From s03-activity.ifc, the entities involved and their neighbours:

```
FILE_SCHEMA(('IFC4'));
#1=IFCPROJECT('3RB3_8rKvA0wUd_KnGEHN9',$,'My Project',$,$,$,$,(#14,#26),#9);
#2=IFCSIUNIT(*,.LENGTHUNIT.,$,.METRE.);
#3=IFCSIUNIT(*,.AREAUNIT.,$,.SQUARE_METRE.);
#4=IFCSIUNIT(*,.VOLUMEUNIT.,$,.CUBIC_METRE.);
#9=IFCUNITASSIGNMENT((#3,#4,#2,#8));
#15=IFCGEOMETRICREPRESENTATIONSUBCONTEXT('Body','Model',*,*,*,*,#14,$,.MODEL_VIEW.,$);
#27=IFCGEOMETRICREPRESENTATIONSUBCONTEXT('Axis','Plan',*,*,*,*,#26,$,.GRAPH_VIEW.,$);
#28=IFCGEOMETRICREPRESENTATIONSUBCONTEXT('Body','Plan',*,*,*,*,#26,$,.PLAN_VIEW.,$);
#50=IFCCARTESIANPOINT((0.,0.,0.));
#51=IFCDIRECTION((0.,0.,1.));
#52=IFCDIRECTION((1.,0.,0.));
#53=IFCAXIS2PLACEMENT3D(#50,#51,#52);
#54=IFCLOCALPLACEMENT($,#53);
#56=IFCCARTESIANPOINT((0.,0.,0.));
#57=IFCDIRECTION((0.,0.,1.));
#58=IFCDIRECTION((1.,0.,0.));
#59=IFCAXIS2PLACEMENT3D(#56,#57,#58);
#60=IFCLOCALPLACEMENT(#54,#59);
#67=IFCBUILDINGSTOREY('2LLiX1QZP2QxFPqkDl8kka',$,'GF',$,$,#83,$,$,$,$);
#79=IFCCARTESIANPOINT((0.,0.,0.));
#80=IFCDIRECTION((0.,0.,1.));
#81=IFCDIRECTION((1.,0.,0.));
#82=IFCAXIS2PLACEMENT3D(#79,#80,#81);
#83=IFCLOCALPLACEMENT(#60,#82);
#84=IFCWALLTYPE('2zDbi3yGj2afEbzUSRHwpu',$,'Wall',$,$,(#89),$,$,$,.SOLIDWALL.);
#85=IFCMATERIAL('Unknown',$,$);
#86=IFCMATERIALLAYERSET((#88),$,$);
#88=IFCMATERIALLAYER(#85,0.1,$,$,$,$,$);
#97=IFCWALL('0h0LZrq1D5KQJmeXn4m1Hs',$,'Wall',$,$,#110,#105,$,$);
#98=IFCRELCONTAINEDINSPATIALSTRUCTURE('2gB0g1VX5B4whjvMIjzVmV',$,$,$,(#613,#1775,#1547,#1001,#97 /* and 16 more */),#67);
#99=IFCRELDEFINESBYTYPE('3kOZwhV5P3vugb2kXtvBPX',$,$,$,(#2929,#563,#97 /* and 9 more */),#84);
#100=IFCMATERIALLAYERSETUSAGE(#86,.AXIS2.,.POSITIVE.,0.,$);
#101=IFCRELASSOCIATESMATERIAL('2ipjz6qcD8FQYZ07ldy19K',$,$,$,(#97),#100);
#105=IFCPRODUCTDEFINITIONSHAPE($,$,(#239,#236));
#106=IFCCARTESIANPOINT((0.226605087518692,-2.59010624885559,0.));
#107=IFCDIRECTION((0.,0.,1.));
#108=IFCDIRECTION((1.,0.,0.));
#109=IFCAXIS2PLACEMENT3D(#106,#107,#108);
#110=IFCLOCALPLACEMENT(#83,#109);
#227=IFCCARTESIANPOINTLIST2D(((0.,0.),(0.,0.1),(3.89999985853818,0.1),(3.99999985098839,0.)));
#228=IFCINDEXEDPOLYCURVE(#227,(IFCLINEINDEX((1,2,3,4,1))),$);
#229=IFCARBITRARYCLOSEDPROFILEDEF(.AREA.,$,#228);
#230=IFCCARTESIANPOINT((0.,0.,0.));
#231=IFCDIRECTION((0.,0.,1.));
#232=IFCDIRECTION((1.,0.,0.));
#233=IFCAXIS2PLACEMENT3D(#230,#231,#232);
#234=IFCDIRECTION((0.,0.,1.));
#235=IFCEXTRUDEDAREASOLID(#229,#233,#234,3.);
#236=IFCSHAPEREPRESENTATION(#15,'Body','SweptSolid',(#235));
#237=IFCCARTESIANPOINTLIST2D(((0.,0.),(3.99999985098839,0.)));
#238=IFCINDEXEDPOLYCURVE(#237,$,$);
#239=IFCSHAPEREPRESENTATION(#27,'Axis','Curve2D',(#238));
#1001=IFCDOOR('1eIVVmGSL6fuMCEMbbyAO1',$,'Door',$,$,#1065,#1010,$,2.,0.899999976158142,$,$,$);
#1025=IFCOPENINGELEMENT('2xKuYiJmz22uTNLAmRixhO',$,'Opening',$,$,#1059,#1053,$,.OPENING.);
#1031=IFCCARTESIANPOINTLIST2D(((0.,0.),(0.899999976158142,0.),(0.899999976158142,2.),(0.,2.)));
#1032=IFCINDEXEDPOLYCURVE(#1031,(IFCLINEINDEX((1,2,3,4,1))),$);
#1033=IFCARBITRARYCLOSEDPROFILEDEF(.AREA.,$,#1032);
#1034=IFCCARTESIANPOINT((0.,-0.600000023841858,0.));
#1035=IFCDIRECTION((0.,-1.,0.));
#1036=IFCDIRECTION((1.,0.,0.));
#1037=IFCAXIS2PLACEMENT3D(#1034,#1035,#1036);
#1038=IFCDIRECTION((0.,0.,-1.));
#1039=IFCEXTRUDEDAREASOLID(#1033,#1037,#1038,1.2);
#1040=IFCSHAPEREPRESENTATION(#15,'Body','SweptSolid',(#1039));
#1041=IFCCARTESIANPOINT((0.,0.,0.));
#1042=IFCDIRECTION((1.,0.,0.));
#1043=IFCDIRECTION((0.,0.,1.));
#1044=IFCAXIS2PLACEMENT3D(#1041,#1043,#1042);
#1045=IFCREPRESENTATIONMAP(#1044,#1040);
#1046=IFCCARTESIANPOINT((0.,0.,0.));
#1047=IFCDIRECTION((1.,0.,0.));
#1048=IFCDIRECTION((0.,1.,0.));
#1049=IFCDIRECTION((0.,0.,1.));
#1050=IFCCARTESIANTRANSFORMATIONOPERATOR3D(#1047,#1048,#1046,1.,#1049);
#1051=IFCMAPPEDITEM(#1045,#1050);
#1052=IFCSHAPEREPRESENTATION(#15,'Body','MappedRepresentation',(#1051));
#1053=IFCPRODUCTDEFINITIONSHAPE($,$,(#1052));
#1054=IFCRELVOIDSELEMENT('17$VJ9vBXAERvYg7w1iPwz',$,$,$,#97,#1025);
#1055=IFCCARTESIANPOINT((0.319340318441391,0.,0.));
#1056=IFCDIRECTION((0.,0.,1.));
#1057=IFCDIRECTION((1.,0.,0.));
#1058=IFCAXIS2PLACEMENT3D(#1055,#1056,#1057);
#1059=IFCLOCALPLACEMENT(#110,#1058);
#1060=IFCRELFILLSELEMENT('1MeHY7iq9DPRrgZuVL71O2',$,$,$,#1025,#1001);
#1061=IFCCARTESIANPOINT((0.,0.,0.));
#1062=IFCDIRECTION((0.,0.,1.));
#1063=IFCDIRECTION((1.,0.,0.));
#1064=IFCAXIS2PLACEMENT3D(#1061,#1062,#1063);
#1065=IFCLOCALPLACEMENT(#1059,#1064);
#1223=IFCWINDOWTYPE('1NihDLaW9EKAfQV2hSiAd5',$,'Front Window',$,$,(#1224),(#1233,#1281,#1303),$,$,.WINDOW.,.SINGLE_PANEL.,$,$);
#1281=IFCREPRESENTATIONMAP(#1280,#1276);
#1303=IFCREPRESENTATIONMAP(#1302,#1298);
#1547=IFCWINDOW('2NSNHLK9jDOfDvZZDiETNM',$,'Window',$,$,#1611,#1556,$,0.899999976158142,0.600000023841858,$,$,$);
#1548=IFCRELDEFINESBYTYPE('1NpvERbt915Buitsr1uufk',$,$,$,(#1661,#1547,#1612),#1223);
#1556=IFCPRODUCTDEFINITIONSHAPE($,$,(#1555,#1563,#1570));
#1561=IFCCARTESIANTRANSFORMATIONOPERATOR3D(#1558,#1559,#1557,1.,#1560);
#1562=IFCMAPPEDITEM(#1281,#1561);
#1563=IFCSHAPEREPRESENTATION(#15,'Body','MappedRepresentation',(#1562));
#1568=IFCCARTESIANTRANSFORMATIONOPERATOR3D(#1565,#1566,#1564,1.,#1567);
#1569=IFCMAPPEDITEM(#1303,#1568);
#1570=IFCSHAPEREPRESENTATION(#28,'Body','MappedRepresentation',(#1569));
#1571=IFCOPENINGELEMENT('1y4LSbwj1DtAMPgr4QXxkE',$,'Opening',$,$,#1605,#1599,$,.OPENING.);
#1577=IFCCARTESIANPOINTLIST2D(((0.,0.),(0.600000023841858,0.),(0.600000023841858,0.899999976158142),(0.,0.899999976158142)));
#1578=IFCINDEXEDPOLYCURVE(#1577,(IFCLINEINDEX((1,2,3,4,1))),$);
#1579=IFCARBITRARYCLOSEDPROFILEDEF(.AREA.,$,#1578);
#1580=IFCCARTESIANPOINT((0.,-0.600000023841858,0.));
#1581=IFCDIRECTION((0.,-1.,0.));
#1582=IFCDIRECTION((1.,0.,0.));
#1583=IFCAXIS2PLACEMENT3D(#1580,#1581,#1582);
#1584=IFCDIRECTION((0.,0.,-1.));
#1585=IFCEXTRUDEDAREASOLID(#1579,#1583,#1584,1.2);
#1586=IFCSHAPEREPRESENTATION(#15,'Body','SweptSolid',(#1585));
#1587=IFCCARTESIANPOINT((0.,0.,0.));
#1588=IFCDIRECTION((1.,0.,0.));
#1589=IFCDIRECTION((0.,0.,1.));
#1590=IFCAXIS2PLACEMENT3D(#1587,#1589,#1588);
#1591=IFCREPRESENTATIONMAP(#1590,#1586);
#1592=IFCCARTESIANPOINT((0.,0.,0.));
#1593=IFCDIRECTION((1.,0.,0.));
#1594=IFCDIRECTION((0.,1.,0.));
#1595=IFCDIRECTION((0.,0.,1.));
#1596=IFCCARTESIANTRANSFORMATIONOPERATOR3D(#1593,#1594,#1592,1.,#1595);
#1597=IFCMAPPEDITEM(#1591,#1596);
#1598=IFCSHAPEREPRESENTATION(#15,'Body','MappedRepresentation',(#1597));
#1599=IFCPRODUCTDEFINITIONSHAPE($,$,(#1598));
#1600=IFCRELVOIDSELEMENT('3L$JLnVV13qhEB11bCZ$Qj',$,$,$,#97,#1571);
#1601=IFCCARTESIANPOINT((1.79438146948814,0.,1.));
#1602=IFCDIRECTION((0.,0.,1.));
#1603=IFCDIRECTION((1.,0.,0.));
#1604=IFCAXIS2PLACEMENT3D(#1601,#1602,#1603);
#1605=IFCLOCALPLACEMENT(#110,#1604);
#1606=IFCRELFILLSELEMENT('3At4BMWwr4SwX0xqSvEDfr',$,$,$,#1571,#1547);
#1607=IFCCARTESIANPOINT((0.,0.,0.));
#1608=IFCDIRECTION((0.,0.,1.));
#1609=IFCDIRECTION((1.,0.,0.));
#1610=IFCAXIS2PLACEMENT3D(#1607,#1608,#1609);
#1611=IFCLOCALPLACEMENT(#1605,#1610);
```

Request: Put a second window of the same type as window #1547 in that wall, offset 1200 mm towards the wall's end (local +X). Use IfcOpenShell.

```python
import ifcopenshell
import ifcopenshell.api.feature
import ifcopenshell.api.geometry
import ifcopenshell.api.root
import ifcopenshell.geom
import ifcopenshell.util.element
import ifcopenshell.util.placement
import ifcopenshell.util.shape
import ifcopenshell.util.unit

model = ifcopenshell.open("s03-activity.ifc")
unit_scale = ifcopenshell.util.unit.calculate_unit_scale(model)
settings = ifcopenshell.geom.settings()


def volume(element):
    """Net volume in cubic metres, openings subtracted."""
    shape = ifcopenshell.geom.create_shape(settings, element)
    return ifcopenshell.util.shape.get_volume(shape.geometry)


window = model.by_id(1547)
opening = window.FillsVoids[0].RelatingOpeningElement
wall = opening.VoidsElements[0].RelatingBuildingElement
before = volume(wall)
shift = ifcopenshell.util.placement.get_local_placement(wall.ObjectPlacement)[:3, 0] * 1.2 / unit_scale

# copy_class copies the void relationship, type, container and properties, but no geometry.
new_opening = ifcopenshell.api.root.copy_class(model, product=opening)
new_opening.Representation = ifcopenshell.util.element.copy_deep(
    model, opening.Representation, exclude=["IfcGeometricRepresentationContext", "IfcRepresentationMap"]
)
new_window = ifcopenshell.api.root.copy_class(model, product=window)
new_window.Representation = ifcopenshell.util.element.copy_deep(
    model, window.Representation, exclude=["IfcGeometricRepresentationContext", "IfcRepresentationMap"]
)
ifcopenshell.api.feature.add_filling(model, opening=new_opening, element=new_window)

for old, new in ((opening, new_opening), (window, new_window)):
    matrix = ifcopenshell.util.placement.get_local_placement(old.ObjectPlacement)
    matrix[:3, 3] += shift
    ifcopenshell.api.geometry.edit_object_placement(model, product=new, matrix=matrix, is_si=False)

after = volume(wall)

print(f"wall volume {before:.3f} -> {after:.3f} m3")

model.write("s03-activity_edited.ifc")
```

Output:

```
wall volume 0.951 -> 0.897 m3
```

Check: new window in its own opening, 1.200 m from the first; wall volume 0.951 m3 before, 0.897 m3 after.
